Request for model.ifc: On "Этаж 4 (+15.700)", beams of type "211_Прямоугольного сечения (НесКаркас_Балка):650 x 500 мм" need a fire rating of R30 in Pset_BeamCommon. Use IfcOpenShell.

First a look at what the model holds.

```python
import ifcopenshell
import ifcopenshell.util.element

model = ifcopenshell.open("model.ifc")
print(model.schema)
storey = next(s for s in model.by_type("IfcBuildingStorey") if s.Name == "Этаж 4 (+15.700)")
beams = [e for e in ifcopenshell.util.element.get_decomposition(storey) if e.is_a("IfcBeam")]
seen = {}
for e in beams:
    element_type = ifcopenshell.util.element.get_type(e)
    key = (element_type.Name if element_type != e and element_type else None, ifcopenshell.util.element.get_pset(e, "Pset_BeamCommon", "FireRating"))
    seen[key] = seen.get(key, 0) + 1
for (name, value), count in sorted(seen.items(), key=str):
    print(count, "x", name, "|", value)
```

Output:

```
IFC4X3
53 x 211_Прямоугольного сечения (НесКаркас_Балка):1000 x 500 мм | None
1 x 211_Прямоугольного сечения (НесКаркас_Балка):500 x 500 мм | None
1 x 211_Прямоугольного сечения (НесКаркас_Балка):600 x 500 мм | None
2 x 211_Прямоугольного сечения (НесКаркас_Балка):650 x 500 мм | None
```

```python
import ifcopenshell
import ifcopenshell.api.pset
import ifcopenshell.util.element

model = ifcopenshell.open("model.ifc")

storey = next(s for s in model.by_type("IfcBuildingStorey") if s.Name == "Этаж 4 (+15.700)")
beams = [e for e in ifcopenshell.util.element.get_decomposition(storey) if e.is_a("IfcBeam")]

count = 0
for e in beams:
    element_type = ifcopenshell.util.element.get_type(e)
    if element_type in (None, e) or element_type.Name != "211_Прямоугольного сечения (НесКаркас_Балка):650 x 500 мм":
        continue
    # add_pset returns the element's existing set when there is one.
    pset = ifcopenshell.api.pset.add_pset(model, product=e, name="Pset_BeamCommon")
    ifcopenshell.api.pset.edit_pset(model, pset=pset, properties={"FireRating": "R30"})
    count += 1

print(count, "beams updated")

model.write("model_updated.ifc")
```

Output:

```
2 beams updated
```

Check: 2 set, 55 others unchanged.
